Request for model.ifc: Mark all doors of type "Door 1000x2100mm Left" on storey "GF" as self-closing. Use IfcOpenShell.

First a look at what the model holds.

```python
import ifcopenshell
import ifcopenshell.util.element

model = ifcopenshell.open("model.ifc")
print(model.schema)
storey = next(s for s in model.by_type("IfcBuildingStorey") if s.Name == "GF")
doors = [e for e in ifcopenshell.util.element.get_decomposition(storey) if e.is_a("IfcDoor")]
seen = {}
for e in doors:
    element_type = ifcopenshell.util.element.get_type(e)
    key = (element_type.Name if element_type != e and element_type else None, ifcopenshell.util.element.get_pset(e, "Pset_DoorCommon", "SelfClosing"))
    seen[key] = seen.get(key, 0) + 1
for (name, value), count in sorted(seen.items(), key=str):
    print(count, "x", name, "|", value)
```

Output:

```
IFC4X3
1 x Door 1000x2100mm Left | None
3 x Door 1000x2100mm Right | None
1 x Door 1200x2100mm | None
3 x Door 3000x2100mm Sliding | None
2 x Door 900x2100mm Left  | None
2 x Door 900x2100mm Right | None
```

```python
import ifcopenshell
import ifcopenshell.api.pset
import ifcopenshell.util.element

model = ifcopenshell.open("model.ifc")

storey = next(s for s in model.by_type("IfcBuildingStorey") if s.Name == "GF")
doors = [e for e in ifcopenshell.util.element.get_decomposition(storey) if e.is_a("IfcDoor")]

count = 0
for e in doors:
    element_type = ifcopenshell.util.element.get_type(e)
    if element_type in (None, e) or element_type.Name != "Door 1000x2100mm Left":
        continue
    # add_pset returns the element's existing set when there is one.
    pset = ifcopenshell.api.pset.add_pset(model, product=e, name="Pset_DoorCommon")
    ifcopenshell.api.pset.edit_pset(model, pset=pset, properties={"SelfClosing": True})
    count += 1

print(count, "doors updated")

model.write("model_edited.ifc")
```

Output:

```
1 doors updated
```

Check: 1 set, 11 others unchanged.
